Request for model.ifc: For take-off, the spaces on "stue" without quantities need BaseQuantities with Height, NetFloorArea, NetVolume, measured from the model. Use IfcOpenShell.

First a look at what the model holds.

```python
import ifcopenshell
import ifcopenshell.util.element
import ifcopenshell.util.unit

model = ifcopenshell.open("model.ifc")
print(model.schema)
for unit_type in ("LENGTHUNIT", "AREAUNIT", "VOLUMEUNIT"):
    print(unit_type, ifcopenshell.util.unit.calculate_unit_scale(model, unit_type))
storey = next(s for s in model.by_type("IfcBuildingStorey") if s.Name == "stue")
spaces = [e for e in ifcopenshell.util.element.get_decomposition(storey) if e.is_a("IfcSpace")]
for e in sorted(spaces, key=lambda e: e.id()):
    print(e.id(), e.is_a(), e.Name, list(ifcopenshell.util.element.get_psets(e, qtos_only=True)), sep=" | ")
```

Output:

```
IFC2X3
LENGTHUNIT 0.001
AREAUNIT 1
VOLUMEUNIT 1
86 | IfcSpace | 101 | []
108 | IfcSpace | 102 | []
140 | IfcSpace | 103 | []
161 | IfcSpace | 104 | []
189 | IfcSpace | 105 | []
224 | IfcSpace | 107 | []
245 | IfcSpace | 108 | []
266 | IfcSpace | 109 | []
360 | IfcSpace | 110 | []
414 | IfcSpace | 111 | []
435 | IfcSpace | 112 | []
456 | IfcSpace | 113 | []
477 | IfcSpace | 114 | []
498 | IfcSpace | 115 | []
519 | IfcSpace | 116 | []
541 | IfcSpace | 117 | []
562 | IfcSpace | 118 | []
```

```python
import ifcopenshell
import ifcopenshell.api.pset
import ifcopenshell.geom
import ifcopenshell.util.element
import ifcopenshell.util.shape
import ifcopenshell.util.unit

model = ifcopenshell.open("model.ifc")
unit_scale = ifcopenshell.util.unit.calculate_unit_scale(model)
area_scale = ifcopenshell.util.unit.calculate_unit_scale(model, "AREAUNIT")
volume_scale = ifcopenshell.util.unit.calculate_unit_scale(model, "VOLUMEUNIT")
settings = ifcopenshell.geom.settings()

storey = next(s for s in model.by_type("IfcBuildingStorey") if s.Name == "stue")
spaces = [e for e in ifcopenshell.util.element.get_decomposition(storey) if e.is_a("IfcSpace")]

for e in sorted(spaces, key=lambda e: e.id()):
    if ifcopenshell.util.element.get_psets(e, qtos_only=True, should_inherit=False):
        continue
    # Geometry comes back in metres, in the element's own axes.
    shape = ifcopenshell.geom.create_shape(settings, e)
    values = {
        "Height": ifcopenshell.util.shape.get_z(shape.geometry) / unit_scale,
        "NetFloorArea": ifcopenshell.util.shape.get_footprint_area(shape.geometry) / area_scale,
        "NetVolume": ifcopenshell.util.shape.get_volume(shape.geometry) / volume_scale,
    }
    qto = ifcopenshell.api.pset.add_qto(model, product=e, name="BaseQuantities")
    ifcopenshell.api.pset.edit_qto(model, qto=qto, properties=values)
    print(e.id(), {k: round(v, 3) for k, v in values.items()})

model.write("model_rev.ifc")
```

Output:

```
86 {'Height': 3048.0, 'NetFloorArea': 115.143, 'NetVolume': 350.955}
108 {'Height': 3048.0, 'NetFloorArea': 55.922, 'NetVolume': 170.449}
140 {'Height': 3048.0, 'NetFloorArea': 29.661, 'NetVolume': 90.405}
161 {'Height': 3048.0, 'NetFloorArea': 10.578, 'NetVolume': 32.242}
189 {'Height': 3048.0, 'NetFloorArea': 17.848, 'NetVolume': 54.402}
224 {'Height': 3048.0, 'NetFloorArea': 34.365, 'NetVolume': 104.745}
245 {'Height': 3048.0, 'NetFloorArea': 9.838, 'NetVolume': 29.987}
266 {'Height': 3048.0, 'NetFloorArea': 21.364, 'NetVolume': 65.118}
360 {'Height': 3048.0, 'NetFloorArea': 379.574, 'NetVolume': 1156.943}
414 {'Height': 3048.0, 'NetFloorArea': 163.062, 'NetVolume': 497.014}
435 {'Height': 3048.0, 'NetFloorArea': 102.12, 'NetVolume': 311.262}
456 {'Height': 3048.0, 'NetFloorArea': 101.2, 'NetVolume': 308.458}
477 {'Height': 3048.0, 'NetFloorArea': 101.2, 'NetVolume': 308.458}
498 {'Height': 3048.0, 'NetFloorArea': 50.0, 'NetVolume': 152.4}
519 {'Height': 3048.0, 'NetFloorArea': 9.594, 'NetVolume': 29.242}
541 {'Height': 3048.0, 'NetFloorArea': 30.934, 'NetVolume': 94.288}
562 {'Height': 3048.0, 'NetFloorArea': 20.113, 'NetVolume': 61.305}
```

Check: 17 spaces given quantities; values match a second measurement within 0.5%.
